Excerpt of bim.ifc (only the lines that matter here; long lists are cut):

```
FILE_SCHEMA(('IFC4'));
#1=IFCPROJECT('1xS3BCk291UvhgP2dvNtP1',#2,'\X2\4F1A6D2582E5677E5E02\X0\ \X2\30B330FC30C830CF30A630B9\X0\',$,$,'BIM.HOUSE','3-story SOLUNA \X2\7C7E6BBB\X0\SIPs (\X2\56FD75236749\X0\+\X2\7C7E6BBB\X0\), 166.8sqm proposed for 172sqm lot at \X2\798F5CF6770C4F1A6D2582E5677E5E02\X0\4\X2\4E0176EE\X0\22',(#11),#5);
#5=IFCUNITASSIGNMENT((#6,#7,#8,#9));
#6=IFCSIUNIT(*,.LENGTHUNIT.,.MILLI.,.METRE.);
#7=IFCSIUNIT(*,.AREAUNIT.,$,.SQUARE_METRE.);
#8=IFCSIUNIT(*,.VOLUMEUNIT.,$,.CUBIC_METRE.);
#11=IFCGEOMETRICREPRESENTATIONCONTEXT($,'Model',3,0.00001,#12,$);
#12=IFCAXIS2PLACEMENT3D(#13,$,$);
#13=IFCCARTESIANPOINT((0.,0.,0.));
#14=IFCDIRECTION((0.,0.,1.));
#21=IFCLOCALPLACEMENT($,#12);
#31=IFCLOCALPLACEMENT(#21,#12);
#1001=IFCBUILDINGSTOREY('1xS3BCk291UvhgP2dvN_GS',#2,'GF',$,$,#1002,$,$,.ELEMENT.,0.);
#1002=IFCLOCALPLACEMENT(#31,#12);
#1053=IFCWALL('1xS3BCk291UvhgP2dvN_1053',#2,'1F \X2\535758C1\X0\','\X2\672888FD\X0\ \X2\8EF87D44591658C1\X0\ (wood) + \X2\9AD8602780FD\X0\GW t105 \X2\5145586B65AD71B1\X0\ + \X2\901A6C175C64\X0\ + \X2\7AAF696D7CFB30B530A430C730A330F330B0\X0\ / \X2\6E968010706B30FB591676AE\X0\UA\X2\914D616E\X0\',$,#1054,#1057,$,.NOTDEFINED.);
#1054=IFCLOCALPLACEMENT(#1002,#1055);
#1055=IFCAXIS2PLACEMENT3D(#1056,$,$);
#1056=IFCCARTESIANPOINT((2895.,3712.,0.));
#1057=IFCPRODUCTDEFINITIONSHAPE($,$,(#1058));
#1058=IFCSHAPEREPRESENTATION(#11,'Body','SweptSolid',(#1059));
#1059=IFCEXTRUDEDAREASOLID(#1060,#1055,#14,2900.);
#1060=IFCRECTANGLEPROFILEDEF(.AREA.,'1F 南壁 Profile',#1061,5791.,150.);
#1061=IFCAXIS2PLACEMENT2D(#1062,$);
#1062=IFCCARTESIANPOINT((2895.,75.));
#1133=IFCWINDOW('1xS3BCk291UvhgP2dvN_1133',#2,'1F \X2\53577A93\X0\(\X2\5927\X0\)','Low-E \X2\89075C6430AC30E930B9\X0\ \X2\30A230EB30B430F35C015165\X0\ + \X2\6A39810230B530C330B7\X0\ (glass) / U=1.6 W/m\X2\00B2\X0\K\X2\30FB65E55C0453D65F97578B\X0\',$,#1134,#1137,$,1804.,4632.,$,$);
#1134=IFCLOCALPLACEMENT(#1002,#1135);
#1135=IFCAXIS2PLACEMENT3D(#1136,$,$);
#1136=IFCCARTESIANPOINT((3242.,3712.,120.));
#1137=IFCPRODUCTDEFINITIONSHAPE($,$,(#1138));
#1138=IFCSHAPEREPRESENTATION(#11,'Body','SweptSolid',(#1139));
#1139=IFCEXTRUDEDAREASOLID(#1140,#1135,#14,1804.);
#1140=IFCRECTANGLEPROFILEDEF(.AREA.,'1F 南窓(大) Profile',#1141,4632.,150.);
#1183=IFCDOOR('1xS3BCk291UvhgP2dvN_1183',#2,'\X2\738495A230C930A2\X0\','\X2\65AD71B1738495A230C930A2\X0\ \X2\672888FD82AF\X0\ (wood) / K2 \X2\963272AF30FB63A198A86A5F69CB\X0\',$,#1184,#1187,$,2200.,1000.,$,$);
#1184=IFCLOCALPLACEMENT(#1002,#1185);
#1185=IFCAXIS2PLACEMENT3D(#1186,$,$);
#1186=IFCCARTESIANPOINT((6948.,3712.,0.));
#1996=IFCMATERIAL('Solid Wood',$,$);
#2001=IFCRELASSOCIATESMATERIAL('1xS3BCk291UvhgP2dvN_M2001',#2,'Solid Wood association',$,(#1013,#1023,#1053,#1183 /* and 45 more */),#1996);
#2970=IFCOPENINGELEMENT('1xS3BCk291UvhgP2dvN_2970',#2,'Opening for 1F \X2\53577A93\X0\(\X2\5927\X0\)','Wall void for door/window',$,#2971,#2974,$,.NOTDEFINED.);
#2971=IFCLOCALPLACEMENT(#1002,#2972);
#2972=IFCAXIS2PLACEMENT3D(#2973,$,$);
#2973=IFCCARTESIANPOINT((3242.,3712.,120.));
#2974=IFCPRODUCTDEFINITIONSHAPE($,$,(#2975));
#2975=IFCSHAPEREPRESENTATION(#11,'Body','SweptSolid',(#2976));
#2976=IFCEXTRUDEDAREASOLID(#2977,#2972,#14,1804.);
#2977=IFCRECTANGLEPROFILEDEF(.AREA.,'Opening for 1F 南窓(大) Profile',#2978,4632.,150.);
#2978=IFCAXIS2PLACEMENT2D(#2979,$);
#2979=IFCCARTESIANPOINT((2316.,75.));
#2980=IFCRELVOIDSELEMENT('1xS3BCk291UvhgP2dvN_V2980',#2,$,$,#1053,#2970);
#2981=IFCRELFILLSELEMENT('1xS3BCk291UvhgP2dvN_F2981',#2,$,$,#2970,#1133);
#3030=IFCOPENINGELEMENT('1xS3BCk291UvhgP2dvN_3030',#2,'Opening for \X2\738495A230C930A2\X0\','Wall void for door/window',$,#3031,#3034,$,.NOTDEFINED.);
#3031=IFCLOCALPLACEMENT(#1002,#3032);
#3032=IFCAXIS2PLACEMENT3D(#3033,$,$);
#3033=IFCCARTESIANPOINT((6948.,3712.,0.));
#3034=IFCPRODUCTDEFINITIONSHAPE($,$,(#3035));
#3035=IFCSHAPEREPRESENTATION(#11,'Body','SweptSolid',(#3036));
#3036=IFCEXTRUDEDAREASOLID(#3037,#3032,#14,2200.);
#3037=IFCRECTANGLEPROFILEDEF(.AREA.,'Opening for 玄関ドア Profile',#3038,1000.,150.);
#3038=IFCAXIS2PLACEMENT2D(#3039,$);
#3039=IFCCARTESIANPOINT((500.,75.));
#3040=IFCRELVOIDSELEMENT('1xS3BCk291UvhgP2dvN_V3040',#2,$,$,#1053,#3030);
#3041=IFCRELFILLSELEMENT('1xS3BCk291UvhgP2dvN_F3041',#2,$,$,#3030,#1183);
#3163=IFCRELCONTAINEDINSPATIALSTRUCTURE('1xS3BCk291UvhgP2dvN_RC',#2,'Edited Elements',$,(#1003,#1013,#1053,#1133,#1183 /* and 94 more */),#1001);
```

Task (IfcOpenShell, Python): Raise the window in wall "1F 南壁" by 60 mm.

```python
import numpy as np
import ifcopenshell
import ifcopenshell.api.geometry
import ifcopenshell.util.placement
import ifcopenshell.util.unit

model = ifcopenshell.open("bim.ifc")
unit_scale = ifcopenshell.util.unit.calculate_unit_scale(model)

window = model.by_guid("1xS3BCk291UvhgP2dvN_1133")
opening = window.FillsVoids[0].RelatingOpeningElement
dz = 60.0

shift = np.array([0.0, 0.0, dz])
# The window is not placed relative to its opening, so move both.
for product in (opening, window):
    matrix = ifcopenshell.util.placement.get_local_placement(product.ObjectPlacement)
    matrix[:3, 3] += shift
    ifcopenshell.api.geometry.edit_object_placement(model, product=product, matrix=matrix, is_si=False)

print(f"moved by {dz * unit_scale:+.3f} m")

model.write("bim-out.ifc")
```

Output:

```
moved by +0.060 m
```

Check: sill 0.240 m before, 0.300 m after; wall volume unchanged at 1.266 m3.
